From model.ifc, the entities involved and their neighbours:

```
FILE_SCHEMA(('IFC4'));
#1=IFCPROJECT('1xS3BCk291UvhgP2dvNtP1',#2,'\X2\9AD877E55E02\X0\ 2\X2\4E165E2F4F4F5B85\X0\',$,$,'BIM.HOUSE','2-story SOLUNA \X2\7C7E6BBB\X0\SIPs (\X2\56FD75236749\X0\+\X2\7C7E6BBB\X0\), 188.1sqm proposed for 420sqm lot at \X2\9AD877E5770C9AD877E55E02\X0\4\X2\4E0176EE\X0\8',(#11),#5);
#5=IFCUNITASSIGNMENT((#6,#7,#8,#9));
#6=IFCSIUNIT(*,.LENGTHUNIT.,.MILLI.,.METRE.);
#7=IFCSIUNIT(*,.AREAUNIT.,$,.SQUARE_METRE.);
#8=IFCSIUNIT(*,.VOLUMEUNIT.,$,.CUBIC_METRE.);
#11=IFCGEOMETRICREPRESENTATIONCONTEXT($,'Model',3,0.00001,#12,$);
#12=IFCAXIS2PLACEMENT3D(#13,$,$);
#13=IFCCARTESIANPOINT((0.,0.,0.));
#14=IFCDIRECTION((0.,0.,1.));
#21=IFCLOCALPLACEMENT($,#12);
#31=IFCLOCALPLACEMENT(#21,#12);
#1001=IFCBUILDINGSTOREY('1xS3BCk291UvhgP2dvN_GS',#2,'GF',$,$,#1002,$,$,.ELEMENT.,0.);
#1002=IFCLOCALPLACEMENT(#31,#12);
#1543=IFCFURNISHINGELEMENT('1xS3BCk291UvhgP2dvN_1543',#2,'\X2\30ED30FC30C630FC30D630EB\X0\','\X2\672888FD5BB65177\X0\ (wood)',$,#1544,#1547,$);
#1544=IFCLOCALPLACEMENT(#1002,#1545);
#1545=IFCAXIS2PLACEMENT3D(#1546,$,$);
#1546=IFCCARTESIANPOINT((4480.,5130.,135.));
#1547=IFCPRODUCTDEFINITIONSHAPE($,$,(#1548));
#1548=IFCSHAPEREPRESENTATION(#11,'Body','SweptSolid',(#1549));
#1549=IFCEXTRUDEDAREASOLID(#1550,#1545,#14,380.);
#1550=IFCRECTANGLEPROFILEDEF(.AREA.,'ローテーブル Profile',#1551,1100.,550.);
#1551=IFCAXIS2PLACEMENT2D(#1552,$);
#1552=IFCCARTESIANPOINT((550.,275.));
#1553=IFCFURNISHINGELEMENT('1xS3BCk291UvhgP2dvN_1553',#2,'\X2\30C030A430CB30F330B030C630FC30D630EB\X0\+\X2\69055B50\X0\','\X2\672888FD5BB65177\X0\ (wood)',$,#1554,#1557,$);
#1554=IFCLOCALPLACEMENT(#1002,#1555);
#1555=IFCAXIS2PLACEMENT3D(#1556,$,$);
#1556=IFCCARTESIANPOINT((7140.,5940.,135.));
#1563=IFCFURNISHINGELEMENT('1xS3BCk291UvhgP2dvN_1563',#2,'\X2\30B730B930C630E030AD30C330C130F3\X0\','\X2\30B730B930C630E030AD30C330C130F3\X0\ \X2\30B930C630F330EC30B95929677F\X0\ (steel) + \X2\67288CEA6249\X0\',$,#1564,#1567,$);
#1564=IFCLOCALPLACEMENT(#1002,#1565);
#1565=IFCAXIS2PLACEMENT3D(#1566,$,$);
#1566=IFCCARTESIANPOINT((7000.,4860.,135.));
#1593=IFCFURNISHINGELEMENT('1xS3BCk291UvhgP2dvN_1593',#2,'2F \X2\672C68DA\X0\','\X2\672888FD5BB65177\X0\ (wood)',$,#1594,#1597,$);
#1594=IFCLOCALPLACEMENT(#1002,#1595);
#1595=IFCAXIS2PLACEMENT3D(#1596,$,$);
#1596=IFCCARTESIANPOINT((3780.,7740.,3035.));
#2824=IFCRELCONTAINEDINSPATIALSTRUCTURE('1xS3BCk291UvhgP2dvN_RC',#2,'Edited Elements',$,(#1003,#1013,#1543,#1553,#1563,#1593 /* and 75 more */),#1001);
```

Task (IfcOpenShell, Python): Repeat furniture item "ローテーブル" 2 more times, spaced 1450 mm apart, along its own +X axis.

```python
import ifcopenshell
import ifcopenshell.api.geometry
import ifcopenshell.api.root
import ifcopenshell.util.element
import ifcopenshell.util.placement

model = ifcopenshell.open("model.ifc")


def reuse_history(source, copy):
    """copy_class also copies each property set's owner history, people and application; keep the originals."""
    for rel in copy.IsDefinedBy:
        if rel.is_a("IfcRelDefinesByProperties") and (history := rel.RelatingPropertyDefinition.OwnerHistory):
            rel.RelatingPropertyDefinition.OwnerHistory = source.OwnerHistory
            ifcopenshell.util.element.remove_deep2(model, history)


source = model.by_id(1543)
base = ifcopenshell.util.placement.get_local_placement(source.ObjectPlacement)
step = base[:3, 0] * 1450.0

for i in range(1, 3):
    copy = ifcopenshell.api.root.copy_class(model, product=source)
    copy.Representation = ifcopenshell.util.element.copy_deep(
        model, source.Representation, exclude=["IfcGeometricRepresentationContext", "IfcRepresentationMap"]
    )
    reuse_history(source, copy)
    matrix = base.copy()
    matrix[:3, 3] += i * step
    print("added at", matrix[:3, 3].round(3) + 0.0)
    ifcopenshell.api.geometry.edit_object_placement(model, product=copy, matrix=matrix, is_si=False)

model.write("model_updated.ifc")
```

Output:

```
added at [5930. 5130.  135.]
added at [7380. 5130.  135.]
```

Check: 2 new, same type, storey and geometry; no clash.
